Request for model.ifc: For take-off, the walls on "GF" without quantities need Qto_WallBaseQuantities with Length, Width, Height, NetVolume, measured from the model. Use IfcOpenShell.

First a look at what the model holds.

```python
import ifcopenshell
import ifcopenshell.util.element
import ifcopenshell.util.unit

model = ifcopenshell.open("model.ifc")
print(model.schema)
for unit_type in ("LENGTHUNIT", "AREAUNIT", "VOLUMEUNIT"):
    print(unit_type, ifcopenshell.util.unit.calculate_unit_scale(model, unit_type))
storey = next(s for s in model.by_type("IfcBuildingStorey") if s.Name == "GF")
walls = [e for e in ifcopenshell.util.element.get_decomposition(storey) if e.is_a("IfcWall")]
for e in sorted(walls, key=lambda e: e.id()):
    print(e.id(), e.is_a(), e.Name, list(ifcopenshell.util.element.get_psets(e, qtos_only=True)), sep=" | ")
```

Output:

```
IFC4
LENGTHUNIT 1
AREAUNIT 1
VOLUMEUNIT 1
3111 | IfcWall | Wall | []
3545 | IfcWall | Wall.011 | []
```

```python
import ifcopenshell
import ifcopenshell.api.pset
import ifcopenshell.geom
import ifcopenshell.util.element
import ifcopenshell.util.shape
import ifcopenshell.util.unit

model = ifcopenshell.open("model.ifc")
unit_scale = ifcopenshell.util.unit.calculate_unit_scale(model)
volume_scale = ifcopenshell.util.unit.calculate_unit_scale(model, "VOLUMEUNIT")
settings = ifcopenshell.geom.settings()

storey = next(s for s in model.by_type("IfcBuildingStorey") if s.Name == "GF")
walls = [e for e in ifcopenshell.util.element.get_decomposition(storey) if e.is_a("IfcWall")]

for e in sorted(walls, key=lambda e: e.id()):
    if ifcopenshell.util.element.get_psets(e, qtos_only=True, should_inherit=False):
        continue
    # Geometry comes back in metres, in the element's own axes.
    shape = ifcopenshell.geom.create_shape(settings, e)
    values = {
        "Length": ifcopenshell.util.shape.get_x(shape.geometry) / unit_scale,
        "Width": ifcopenshell.util.shape.get_y(shape.geometry) / unit_scale,
        "Height": ifcopenshell.util.shape.get_z(shape.geometry) / unit_scale,
        "NetVolume": ifcopenshell.util.shape.get_volume(shape.geometry) / volume_scale,
    }
    qto = ifcopenshell.api.pset.add_qto(model, product=e, name="Qto_WallBaseQuantities")
    ifcopenshell.api.pset.edit_qto(model, qto=qto, properties=values)
    print(e.id(), {k: round(v, 3) for k, v in values.items()})

model.write("model_edited.ifc")
```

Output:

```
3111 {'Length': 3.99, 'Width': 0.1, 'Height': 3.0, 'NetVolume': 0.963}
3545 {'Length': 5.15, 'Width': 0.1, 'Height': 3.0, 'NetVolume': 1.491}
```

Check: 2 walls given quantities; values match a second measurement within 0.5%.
